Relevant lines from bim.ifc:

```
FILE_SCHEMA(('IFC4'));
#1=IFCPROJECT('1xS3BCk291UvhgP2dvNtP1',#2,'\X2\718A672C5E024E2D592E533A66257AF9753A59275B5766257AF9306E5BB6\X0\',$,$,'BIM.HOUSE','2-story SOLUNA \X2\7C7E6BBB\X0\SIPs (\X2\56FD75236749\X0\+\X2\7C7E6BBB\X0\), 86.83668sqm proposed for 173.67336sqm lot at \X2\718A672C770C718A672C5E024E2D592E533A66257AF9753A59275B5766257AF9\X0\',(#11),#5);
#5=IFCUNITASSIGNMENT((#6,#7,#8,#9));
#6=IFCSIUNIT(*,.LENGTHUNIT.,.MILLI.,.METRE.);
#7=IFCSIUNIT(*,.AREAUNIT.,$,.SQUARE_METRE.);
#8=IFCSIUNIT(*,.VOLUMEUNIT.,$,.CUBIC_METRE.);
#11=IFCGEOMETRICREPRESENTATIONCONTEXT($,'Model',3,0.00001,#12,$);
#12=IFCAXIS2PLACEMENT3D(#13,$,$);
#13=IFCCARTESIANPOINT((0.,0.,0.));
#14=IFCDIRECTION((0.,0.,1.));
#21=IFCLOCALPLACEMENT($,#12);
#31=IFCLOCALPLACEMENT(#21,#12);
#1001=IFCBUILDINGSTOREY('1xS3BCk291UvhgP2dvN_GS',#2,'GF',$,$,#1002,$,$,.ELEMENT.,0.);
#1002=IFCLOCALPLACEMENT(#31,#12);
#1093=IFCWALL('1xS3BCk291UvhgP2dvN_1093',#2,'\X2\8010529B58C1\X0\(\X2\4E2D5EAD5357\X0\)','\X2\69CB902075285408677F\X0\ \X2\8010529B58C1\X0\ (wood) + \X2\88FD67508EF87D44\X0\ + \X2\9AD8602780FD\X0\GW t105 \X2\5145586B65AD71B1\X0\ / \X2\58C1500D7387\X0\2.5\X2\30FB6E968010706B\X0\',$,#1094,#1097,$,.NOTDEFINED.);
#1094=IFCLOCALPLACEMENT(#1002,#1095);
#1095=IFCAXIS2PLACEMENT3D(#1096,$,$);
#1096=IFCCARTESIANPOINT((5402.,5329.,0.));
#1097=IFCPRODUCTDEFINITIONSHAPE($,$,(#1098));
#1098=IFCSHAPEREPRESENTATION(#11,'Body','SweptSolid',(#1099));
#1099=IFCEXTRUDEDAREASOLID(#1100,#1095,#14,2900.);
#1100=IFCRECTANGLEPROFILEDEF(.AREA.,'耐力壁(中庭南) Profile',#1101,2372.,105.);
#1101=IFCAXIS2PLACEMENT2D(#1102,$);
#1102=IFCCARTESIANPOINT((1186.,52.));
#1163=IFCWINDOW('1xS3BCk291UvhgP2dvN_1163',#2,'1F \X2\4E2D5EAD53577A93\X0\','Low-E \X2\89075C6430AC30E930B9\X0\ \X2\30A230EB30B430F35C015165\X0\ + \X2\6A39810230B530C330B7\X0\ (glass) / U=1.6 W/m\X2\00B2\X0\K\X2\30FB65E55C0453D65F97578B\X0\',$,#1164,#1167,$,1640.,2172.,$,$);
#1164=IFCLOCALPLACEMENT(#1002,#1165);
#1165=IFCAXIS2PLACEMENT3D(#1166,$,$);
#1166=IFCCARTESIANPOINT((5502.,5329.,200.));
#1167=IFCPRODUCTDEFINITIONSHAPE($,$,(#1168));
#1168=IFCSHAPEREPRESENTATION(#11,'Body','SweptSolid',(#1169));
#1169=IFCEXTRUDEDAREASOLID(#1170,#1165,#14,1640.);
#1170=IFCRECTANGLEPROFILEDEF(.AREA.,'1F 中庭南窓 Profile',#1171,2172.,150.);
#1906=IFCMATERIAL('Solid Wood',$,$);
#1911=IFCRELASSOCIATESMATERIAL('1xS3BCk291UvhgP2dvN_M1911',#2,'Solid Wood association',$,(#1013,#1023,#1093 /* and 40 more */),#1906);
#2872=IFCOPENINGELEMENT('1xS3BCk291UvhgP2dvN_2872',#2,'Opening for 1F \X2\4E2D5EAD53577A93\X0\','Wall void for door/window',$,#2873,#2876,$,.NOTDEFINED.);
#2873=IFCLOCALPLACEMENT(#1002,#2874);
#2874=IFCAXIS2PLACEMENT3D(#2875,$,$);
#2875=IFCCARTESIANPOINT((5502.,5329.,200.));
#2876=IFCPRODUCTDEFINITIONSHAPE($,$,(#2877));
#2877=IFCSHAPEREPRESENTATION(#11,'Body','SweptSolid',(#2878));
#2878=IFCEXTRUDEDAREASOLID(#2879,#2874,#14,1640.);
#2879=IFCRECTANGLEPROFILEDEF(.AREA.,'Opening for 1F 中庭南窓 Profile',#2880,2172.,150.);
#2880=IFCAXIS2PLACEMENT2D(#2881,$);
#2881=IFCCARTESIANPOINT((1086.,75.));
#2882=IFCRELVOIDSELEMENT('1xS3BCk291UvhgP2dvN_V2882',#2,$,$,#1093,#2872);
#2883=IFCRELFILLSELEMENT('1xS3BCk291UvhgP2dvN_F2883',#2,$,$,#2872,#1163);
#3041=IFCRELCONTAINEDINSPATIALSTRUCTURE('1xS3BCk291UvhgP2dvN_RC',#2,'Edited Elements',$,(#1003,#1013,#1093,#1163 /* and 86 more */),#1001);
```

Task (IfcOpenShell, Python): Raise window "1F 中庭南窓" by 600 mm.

```python
import numpy as np
import ifcopenshell
import ifcopenshell.api.geometry
import ifcopenshell.util.placement
import ifcopenshell.util.unit

model = ifcopenshell.open("bim.ifc")
unit_scale = ifcopenshell.util.unit.calculate_unit_scale(model)

window = model.by_guid("1xS3BCk291UvhgP2dvN_1163")
opening = window.FillsVoids[0].RelatingOpeningElement
dz = 0.6 / unit_scale

shift = np.array([0.0, 0.0, dz])
# The window is not placed relative to its opening, so move both.
for product in (opening, window):
    matrix = ifcopenshell.util.placement.get_local_placement(product.ObjectPlacement)
    matrix[:3, 3] += shift
    ifcopenshell.api.geometry.edit_object_placement(model, product=product, matrix=matrix, is_si=False)

print(f"moved by {dz * unit_scale:+.3f} m")

model.write("bim_edited.ifc")
```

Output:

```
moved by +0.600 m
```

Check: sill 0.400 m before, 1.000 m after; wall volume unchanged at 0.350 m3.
